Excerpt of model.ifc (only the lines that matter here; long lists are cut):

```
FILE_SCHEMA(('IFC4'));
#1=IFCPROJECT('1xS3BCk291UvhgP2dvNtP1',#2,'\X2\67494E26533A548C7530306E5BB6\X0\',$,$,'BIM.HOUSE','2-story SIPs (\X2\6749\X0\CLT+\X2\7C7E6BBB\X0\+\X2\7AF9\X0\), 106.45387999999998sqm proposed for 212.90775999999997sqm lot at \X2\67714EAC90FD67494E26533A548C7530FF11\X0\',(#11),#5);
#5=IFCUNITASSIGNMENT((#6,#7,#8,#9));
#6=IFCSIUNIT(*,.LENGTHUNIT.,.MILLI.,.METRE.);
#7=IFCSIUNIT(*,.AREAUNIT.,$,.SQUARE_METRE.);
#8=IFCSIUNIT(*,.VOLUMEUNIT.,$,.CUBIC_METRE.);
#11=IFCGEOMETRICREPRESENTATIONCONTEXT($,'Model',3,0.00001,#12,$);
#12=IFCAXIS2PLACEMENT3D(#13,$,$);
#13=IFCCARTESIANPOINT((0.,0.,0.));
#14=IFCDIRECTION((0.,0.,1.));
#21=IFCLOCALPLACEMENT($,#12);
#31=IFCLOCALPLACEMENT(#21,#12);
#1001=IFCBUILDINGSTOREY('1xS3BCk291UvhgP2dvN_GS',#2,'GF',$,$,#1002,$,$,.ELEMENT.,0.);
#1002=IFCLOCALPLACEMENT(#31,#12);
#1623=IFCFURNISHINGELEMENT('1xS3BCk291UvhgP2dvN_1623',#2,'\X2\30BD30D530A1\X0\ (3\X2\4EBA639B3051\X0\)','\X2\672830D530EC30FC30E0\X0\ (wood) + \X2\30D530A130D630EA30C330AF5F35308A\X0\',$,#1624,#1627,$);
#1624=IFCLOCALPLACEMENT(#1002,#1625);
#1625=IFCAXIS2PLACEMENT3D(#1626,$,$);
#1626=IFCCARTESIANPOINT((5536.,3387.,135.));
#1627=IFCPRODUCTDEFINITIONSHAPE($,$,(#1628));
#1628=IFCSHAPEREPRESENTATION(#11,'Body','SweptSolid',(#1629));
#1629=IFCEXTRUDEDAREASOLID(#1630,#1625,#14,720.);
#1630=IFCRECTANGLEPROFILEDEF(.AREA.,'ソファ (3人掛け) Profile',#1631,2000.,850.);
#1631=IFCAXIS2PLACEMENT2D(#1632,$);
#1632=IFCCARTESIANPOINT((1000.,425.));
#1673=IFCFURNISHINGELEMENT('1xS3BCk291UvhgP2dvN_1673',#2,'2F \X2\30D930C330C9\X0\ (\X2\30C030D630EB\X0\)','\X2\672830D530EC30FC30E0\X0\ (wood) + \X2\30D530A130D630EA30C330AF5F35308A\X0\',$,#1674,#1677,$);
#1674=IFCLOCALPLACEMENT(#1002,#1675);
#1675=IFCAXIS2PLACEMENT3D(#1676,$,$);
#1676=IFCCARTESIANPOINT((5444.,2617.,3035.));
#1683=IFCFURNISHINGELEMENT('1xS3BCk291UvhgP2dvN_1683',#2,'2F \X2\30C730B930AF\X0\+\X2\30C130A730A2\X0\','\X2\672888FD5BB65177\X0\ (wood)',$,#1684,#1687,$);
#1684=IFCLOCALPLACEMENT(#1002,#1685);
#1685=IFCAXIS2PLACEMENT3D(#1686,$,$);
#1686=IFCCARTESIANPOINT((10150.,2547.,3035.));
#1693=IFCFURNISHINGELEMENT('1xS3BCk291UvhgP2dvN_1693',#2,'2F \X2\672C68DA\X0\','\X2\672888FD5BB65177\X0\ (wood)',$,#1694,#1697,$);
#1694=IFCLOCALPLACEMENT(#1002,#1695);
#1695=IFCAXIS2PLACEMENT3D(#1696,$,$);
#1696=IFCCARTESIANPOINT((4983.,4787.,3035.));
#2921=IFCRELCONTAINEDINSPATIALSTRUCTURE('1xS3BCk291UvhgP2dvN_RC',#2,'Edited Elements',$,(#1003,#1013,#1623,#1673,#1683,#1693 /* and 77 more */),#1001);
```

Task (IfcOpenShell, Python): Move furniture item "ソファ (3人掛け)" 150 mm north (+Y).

```python
import ifcopenshell
import ifcopenshell.api.geometry
import ifcopenshell.util.placement
import ifcopenshell.util.unit

model = ifcopenshell.open("model.ifc")
unit_scale = ifcopenshell.util.unit.calculate_unit_scale(model)

item = model.by_id(1623)
matrix = ifcopenshell.util.placement.get_local_placement(item.ObjectPlacement)
matrix[1, 3] += 0.15 / unit_scale
ifcopenshell.api.geometry.edit_object_placement(model, product=item, matrix=matrix, is_si=False)

print(ifcopenshell.util.placement.get_local_placement(item.ObjectPlacement).round(3) + 0.0)

model.write("model-out.ifc")
```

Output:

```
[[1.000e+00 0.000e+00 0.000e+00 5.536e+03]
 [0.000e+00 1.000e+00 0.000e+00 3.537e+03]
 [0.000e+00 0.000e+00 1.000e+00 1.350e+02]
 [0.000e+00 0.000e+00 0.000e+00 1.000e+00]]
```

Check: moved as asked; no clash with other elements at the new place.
